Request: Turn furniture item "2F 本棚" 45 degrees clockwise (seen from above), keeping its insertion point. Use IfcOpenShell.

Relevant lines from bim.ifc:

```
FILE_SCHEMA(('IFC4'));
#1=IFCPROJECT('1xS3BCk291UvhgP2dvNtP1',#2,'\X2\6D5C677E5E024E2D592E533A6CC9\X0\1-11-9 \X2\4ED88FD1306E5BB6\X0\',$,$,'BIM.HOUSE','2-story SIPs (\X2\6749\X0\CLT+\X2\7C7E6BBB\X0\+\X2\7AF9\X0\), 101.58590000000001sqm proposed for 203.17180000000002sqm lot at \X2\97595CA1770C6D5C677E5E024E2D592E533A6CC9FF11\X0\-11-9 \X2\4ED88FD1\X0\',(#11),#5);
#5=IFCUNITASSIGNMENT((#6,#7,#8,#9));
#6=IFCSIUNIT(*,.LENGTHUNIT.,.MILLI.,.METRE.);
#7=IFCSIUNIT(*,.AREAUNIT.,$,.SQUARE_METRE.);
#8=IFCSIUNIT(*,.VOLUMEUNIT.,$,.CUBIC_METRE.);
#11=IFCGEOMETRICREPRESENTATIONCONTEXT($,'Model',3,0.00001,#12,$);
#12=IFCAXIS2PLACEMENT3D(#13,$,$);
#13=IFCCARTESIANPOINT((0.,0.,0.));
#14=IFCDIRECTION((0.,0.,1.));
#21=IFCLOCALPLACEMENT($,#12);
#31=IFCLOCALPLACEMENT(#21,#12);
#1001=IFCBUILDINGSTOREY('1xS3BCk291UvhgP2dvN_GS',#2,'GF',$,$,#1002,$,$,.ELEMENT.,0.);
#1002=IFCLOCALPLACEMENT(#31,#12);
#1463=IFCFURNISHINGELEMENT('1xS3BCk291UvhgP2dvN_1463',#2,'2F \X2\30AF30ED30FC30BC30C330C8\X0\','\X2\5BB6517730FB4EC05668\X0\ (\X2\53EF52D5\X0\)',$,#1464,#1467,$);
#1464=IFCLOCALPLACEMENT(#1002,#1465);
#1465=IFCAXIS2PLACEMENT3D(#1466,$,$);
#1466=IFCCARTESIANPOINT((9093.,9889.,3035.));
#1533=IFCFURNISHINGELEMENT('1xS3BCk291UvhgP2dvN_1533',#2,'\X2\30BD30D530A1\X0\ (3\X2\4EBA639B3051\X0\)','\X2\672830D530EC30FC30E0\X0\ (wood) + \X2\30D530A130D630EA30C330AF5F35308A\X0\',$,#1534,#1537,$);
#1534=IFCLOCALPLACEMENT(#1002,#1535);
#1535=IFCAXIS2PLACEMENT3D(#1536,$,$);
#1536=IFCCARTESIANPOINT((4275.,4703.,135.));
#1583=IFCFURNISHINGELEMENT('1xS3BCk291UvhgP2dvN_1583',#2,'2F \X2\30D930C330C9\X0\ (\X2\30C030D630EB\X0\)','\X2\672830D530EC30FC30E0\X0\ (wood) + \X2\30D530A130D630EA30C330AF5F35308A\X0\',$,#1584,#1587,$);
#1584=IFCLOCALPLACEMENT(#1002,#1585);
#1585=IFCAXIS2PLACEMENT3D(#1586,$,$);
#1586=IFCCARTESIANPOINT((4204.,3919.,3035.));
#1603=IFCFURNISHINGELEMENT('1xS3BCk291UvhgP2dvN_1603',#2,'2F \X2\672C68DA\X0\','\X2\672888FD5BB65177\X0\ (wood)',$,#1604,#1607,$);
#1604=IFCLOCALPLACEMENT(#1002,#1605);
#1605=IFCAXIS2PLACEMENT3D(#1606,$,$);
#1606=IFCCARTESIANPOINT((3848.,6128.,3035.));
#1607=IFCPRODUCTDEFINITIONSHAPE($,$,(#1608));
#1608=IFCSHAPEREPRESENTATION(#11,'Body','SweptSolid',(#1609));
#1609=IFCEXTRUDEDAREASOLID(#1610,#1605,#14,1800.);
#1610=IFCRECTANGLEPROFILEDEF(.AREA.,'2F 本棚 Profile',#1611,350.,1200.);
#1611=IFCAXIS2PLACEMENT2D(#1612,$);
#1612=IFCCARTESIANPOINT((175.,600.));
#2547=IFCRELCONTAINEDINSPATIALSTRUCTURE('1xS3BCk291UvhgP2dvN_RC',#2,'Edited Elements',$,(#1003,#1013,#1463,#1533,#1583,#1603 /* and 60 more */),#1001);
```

```python
import ifcopenshell
import ifcopenshell.api.geometry
import ifcopenshell.util.placement

model = ifcopenshell.open("bim.ifc")

item = model.by_guid("1xS3BCk291UvhgP2dvN_1603")
matrix = ifcopenshell.util.placement.get_local_placement(item.ObjectPlacement)
matrix = matrix @ ifcopenshell.util.placement.rotation(-45, "Z")
ifcopenshell.api.geometry.edit_object_placement(model, product=item, matrix=matrix, is_si=False)

print(ifcopenshell.util.placement.get_local_placement(item.ObjectPlacement).round(3) + 0.0)

model.write("bim_edited.ifc")
```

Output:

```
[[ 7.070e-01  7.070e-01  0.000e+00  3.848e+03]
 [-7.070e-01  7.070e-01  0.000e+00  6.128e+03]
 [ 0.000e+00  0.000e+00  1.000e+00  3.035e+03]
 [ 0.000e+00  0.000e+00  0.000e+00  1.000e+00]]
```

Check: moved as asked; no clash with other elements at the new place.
